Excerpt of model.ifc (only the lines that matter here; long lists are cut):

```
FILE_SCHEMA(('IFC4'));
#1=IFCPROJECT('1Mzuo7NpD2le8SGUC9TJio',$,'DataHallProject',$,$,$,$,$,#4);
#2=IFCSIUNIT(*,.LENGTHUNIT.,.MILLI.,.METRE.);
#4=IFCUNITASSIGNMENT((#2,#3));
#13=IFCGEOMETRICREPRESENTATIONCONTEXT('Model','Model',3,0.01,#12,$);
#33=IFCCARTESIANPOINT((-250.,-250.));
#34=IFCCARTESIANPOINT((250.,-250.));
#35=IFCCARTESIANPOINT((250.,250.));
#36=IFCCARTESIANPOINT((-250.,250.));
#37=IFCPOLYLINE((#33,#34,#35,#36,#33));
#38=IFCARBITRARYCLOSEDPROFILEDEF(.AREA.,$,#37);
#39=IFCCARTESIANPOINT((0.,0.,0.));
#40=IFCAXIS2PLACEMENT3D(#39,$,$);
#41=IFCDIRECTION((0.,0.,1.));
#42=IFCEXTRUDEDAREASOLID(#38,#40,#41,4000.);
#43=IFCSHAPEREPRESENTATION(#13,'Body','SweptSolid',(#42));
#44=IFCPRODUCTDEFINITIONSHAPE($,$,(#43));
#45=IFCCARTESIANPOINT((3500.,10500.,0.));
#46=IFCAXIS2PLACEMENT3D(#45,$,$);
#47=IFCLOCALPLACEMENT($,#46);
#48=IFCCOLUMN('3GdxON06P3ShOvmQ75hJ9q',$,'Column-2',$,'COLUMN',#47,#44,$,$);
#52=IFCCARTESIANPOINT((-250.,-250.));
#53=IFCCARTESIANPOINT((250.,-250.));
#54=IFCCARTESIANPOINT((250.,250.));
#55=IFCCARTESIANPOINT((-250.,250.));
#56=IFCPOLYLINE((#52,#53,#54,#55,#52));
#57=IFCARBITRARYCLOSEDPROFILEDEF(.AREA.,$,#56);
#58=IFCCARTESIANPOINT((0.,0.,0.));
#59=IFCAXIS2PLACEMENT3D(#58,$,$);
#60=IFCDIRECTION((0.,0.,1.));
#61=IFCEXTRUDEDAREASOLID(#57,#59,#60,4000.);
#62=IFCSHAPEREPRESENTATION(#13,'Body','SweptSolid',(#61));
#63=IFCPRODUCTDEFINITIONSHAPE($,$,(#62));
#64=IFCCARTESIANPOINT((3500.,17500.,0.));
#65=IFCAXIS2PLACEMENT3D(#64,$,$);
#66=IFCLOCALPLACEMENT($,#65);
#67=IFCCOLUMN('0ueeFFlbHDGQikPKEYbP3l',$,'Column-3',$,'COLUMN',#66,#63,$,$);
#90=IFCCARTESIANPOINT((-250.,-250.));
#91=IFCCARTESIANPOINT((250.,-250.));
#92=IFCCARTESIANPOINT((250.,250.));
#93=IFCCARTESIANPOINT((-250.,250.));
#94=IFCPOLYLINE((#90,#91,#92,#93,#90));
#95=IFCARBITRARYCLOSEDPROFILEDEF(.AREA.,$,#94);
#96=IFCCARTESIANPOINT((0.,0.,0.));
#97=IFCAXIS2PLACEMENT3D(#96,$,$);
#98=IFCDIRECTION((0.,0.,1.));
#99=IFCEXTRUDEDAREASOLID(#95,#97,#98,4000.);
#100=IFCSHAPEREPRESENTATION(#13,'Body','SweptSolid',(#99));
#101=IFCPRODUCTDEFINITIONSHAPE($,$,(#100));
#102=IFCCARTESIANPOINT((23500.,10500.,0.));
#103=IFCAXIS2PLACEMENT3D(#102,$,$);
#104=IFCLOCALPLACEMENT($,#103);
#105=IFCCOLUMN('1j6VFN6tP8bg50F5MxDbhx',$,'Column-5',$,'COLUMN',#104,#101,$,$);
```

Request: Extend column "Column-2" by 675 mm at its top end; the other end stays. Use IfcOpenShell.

```python
import ifcopenshell
import ifcopenshell.util.unit

model = ifcopenshell.open("model.ifc")
unit_scale = ifcopenshell.util.unit.calculate_unit_scale(model)

member = model.by_id(48)
change = 0.675 / unit_scale

# The extrusion runs towards the end named, so only its depth changes.
body = next(r for r in member.Representation.Representations if r.RepresentationIdentifier == "Body")
solid = body.Items[0]
old_length = solid.Depth
solid.Depth += change

print(f"length {old_length:g} -> {solid.Depth:g}")

model.write("model_v2.ifc")
```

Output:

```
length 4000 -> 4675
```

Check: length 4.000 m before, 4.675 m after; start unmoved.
